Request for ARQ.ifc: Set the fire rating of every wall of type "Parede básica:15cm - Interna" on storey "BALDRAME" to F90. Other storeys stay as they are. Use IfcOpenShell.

First a look at what the model holds.

```python
import ifcopenshell
import ifcopenshell.util.element

model = ifcopenshell.open("ARQ.ifc")
print(model.schema)
storey = next(s for s in model.by_type("IfcBuildingStorey") if s.Name == "BALDRAME")
walls = [e for e in ifcopenshell.util.element.get_decomposition(storey) if e.is_a("IfcWall")]
seen = {}
for e in walls:
    element_type = ifcopenshell.util.element.get_type(e)
    key = (element_type.Name if element_type != e and element_type else None, ifcopenshell.util.element.get_pset(e, "Pset_WallCommon", "FireRating"))
    seen[key] = seen.get(key, 0) + 1
for (name, value), count in sorted(seen.items(), key=str):
    print(count, "x", name, "|", value)
```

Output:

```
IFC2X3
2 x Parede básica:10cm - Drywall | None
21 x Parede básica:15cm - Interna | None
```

```python
import ifcopenshell
import ifcopenshell.api.pset
import ifcopenshell.util.element

model = ifcopenshell.open("ARQ.ifc")

storey = next(s for s in model.by_type("IfcBuildingStorey") if s.Name == "BALDRAME")
walls = [e for e in ifcopenshell.util.element.get_decomposition(storey) if e.is_a("IfcWall")]

count = 0
for e in walls:
    element_type = ifcopenshell.util.element.get_type(e)
    if element_type in (None, e) or element_type.Name != "Parede básica:15cm - Interna":
        continue
    # add_pset returns the element's existing set when there is one.
    pset = ifcopenshell.api.pset.add_pset(model, product=e, name="Pset_WallCommon")
    ifcopenshell.api.pset.edit_pset(model, pset=pset, properties={"FireRating": "F90"})
    count += 1

print(count, "walls updated")

model.write("ARQ_v2.ifc")
```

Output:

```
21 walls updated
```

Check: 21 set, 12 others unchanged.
